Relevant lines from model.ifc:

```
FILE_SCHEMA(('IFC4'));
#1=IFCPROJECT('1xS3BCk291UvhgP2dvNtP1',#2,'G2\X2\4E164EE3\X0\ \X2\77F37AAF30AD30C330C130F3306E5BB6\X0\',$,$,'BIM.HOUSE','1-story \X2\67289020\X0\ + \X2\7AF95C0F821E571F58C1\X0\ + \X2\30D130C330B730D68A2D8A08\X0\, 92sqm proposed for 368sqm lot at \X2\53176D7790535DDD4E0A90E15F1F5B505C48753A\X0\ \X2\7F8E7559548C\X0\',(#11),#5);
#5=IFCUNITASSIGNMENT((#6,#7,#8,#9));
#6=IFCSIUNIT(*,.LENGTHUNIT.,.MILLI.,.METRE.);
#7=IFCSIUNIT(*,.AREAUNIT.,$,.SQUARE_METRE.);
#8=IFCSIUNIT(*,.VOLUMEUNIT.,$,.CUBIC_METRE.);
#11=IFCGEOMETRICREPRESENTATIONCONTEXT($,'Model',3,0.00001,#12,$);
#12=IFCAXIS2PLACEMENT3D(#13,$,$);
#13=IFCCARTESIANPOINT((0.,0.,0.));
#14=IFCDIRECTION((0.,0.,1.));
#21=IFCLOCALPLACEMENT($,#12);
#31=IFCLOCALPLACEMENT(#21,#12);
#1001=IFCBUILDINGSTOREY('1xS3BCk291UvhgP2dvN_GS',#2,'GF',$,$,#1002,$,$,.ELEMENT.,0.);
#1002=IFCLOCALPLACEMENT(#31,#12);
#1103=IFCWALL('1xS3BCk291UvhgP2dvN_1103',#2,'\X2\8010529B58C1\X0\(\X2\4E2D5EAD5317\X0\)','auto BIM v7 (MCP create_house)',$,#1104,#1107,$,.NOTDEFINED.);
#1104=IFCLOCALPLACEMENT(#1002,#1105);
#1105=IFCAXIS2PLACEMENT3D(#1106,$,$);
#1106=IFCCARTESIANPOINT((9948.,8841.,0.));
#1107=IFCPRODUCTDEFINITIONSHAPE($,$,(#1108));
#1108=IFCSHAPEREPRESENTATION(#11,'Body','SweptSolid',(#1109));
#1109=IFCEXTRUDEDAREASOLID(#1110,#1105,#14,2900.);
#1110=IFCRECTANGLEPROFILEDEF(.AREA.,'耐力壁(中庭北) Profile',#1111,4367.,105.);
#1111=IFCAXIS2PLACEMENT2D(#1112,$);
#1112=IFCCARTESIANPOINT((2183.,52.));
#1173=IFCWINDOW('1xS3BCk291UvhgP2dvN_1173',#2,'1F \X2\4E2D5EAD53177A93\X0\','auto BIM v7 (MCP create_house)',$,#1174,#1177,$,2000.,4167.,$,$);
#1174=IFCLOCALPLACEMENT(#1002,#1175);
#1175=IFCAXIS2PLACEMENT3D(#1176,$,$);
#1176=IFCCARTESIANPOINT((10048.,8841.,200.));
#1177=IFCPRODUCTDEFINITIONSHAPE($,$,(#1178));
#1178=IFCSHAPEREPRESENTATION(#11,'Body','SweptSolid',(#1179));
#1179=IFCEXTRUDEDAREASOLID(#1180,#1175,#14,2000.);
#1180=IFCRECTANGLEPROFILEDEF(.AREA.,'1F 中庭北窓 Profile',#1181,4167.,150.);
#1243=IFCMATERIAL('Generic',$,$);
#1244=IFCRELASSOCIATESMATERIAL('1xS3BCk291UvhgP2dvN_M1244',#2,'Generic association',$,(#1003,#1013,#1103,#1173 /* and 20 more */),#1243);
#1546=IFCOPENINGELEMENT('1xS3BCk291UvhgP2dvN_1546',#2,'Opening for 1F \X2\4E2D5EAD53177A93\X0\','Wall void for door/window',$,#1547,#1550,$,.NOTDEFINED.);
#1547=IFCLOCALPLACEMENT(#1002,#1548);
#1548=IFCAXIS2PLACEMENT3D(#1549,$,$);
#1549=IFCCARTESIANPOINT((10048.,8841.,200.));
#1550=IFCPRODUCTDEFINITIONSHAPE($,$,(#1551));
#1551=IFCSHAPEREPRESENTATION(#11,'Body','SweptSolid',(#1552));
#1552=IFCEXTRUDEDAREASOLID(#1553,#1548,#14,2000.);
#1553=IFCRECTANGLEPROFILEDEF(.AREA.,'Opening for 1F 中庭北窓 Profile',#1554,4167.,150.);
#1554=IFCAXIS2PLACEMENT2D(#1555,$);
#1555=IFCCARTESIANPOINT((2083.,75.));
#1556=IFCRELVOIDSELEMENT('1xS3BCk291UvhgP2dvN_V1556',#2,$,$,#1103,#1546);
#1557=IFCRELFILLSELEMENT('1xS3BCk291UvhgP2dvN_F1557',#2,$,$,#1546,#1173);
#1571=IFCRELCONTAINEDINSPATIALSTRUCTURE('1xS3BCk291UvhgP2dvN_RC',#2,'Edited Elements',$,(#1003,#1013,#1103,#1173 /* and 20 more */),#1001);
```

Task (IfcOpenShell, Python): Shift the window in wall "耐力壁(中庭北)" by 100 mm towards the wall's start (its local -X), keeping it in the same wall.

```python
import ifcopenshell
import ifcopenshell.api.geometry
import ifcopenshell.util.placement
import ifcopenshell.util.unit

model = ifcopenshell.open("model.ifc")
unit_scale = ifcopenshell.util.unit.calculate_unit_scale(model)

window = model.by_guid("1xS3BCk291UvhgP2dvN_1173")
opening = window.FillsVoids[0].RelatingOpeningElement
wall = opening.VoidsElements[0].RelatingBuildingElement

wall_matrix = ifcopenshell.util.placement.get_local_placement(wall.ObjectPlacement)
shift = wall_matrix[:3, 0] * -0.1 / unit_scale
before = ifcopenshell.util.placement.get_local_placement(window.ObjectPlacement)[:3, 3].copy()

# The window is not placed relative to its opening, so move both.
for product in (opening, window):
    matrix = ifcopenshell.util.placement.get_local_placement(product.ObjectPlacement)
    matrix[:3, 3] += shift
    ifcopenshell.api.geometry.edit_object_placement(model, product=product, matrix=matrix, is_si=False)

after = ifcopenshell.util.placement.get_local_placement(window.ObjectPlacement)[:3, 3]
print("window moved by", (after - before).round(3) + 0.0)

model.write("model_edited.ifc")
```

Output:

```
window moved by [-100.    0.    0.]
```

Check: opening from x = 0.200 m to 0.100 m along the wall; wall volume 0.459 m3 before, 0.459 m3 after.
